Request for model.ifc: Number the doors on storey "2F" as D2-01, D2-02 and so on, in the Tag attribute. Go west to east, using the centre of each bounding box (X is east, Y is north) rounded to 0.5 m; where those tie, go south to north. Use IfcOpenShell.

First a look at what the model holds.

```python
import ifcopenshell
import ifcopenshell.util.element
import ifcopenshell.util.placement

model = ifcopenshell.open("model.ifc")
print(model.schema)
storey = next(s for s in model.by_type("IfcBuildingStorey") if s.Name == "2F")
doors = [e for e in ifcopenshell.util.element.get_decomposition(storey) if e.is_a("IfcDoor")]
for e in sorted(doors, key=lambda e: e.id()):
    origin = ifcopenshell.util.placement.get_local_placement(e.ObjectPlacement)[:3, 3]
    print(e.id(), e.Tag, e.Name, origin.round(2) + 0.0, sep=" | ")
```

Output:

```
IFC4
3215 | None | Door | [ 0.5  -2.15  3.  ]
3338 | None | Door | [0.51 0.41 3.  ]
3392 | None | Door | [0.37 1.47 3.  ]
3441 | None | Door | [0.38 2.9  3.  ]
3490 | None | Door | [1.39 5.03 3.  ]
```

```python
import ifcopenshell
import ifcopenshell.geom
import ifcopenshell.util.element
import ifcopenshell.util.shape

model = ifcopenshell.open("model.ifc")
settings = ifcopenshell.geom.settings()
settings.set("use-world-coords", True)


def centre(element):
    shape = ifcopenshell.geom.create_shape(settings, element)
    return ifcopenshell.util.shape.get_bbox_centroid(shape.geometry)


storey = next(s for s in model.by_type("IfcBuildingStorey") if s.Name == "2F")
doors = [e for e in ifcopenshell.util.element.get_decomposition(storey) if e.is_a("IfcDoor")]

# Insertion points can sit at a corner or the storey origin, so sort by the geometry (in metres).
centres = {e: centre(e) for e in doors}
doors.sort(key=lambda e: (round(centres[e][0] / 0.5), centres[e][1]))

for i, e in enumerate(doors, start=1):
    number = f"D2-{i:02d}"
    e.Tag = number
    print(e.id(), number)

model.write("model_v2.ifc")
```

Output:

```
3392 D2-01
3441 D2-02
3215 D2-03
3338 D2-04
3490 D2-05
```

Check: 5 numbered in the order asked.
